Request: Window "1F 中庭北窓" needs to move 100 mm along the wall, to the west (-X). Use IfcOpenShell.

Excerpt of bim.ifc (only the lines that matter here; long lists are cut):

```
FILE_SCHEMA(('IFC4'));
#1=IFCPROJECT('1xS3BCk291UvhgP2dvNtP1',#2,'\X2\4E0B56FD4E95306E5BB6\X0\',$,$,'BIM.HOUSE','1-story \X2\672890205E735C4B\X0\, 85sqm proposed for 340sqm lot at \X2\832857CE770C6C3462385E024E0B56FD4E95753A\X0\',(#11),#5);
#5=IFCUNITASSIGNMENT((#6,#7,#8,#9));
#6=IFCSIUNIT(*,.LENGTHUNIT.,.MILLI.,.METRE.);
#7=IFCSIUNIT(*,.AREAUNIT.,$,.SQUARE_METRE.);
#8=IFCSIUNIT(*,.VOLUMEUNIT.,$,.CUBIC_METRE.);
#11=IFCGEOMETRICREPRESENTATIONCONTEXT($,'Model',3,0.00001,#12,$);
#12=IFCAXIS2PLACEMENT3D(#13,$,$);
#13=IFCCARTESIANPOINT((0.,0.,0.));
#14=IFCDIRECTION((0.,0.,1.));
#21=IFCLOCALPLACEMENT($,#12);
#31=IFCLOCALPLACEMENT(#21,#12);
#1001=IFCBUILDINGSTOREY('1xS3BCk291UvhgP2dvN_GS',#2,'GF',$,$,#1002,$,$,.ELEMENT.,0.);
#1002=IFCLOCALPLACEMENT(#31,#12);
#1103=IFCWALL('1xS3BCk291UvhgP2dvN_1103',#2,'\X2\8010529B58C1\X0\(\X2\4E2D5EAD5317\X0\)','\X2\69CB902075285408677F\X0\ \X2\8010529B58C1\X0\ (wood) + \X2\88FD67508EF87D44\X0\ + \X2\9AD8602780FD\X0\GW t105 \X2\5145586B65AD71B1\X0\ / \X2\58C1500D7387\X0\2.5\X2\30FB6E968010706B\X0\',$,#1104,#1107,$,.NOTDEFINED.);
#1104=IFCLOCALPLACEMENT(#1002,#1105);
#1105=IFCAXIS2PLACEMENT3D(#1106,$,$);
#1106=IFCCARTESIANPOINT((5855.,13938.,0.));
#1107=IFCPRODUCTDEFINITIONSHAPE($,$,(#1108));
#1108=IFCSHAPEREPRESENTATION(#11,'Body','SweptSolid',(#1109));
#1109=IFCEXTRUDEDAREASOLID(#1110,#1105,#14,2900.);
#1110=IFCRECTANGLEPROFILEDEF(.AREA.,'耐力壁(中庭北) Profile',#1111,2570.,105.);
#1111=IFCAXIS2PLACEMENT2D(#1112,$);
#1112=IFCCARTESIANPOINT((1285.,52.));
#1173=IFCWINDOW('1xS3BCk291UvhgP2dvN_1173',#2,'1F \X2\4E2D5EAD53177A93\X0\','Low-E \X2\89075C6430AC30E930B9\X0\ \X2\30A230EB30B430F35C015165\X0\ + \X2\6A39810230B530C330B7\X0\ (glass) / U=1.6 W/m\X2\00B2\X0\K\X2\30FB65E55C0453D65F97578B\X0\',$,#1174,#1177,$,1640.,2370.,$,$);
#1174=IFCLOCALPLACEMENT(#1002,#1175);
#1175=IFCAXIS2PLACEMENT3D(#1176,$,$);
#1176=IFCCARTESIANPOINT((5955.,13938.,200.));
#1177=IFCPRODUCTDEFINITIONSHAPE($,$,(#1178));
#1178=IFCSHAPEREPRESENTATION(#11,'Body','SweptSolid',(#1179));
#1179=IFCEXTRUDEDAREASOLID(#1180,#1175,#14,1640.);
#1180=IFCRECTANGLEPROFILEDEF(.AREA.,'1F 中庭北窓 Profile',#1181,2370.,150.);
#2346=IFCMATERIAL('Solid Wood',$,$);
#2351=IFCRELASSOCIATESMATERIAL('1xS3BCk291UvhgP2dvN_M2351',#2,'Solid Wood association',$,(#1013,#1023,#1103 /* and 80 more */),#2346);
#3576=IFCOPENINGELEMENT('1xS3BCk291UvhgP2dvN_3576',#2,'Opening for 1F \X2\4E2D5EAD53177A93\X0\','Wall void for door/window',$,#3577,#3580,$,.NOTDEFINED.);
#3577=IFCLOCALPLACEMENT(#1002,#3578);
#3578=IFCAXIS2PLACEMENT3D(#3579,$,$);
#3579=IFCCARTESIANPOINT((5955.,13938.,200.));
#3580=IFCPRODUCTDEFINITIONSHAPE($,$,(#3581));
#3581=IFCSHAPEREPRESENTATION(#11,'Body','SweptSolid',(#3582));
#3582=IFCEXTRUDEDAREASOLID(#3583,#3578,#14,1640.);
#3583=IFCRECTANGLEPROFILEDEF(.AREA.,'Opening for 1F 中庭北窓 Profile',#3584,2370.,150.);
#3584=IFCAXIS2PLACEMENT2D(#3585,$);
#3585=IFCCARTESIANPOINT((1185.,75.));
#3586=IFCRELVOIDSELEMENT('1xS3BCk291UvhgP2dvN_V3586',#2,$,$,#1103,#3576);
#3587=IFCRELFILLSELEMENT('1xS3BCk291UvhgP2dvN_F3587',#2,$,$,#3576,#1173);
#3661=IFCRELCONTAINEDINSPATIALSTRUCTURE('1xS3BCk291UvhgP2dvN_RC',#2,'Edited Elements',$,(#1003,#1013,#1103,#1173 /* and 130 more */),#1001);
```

```python
import ifcopenshell
import ifcopenshell.api.geometry
import ifcopenshell.util.placement

model = ifcopenshell.open("bim.ifc")

window = model.by_id(1173)
opening = window.FillsVoids[0].RelatingOpeningElement
wall = opening.VoidsElements[0].RelatingBuildingElement

wall_matrix = ifcopenshell.util.placement.get_local_placement(wall.ObjectPlacement)
shift = wall_matrix[:3, 0] * -100.0
before = ifcopenshell.util.placement.get_local_placement(window.ObjectPlacement)[:3, 3].copy()

# The window is not placed relative to its opening, so move both.
for product in (opening, window):
    matrix = ifcopenshell.util.placement.get_local_placement(product.ObjectPlacement)
    matrix[:3, 3] += shift
    ifcopenshell.api.geometry.edit_object_placement(model, product=product, matrix=matrix, is_si=False)

after = ifcopenshell.util.placement.get_local_placement(window.ObjectPlacement)[:3, 3]
print("window moved by", (after - before).round(3) + 0.0)

model.write("bim_rev.ifc")
```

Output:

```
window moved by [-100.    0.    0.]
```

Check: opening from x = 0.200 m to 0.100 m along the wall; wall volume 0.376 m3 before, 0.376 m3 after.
